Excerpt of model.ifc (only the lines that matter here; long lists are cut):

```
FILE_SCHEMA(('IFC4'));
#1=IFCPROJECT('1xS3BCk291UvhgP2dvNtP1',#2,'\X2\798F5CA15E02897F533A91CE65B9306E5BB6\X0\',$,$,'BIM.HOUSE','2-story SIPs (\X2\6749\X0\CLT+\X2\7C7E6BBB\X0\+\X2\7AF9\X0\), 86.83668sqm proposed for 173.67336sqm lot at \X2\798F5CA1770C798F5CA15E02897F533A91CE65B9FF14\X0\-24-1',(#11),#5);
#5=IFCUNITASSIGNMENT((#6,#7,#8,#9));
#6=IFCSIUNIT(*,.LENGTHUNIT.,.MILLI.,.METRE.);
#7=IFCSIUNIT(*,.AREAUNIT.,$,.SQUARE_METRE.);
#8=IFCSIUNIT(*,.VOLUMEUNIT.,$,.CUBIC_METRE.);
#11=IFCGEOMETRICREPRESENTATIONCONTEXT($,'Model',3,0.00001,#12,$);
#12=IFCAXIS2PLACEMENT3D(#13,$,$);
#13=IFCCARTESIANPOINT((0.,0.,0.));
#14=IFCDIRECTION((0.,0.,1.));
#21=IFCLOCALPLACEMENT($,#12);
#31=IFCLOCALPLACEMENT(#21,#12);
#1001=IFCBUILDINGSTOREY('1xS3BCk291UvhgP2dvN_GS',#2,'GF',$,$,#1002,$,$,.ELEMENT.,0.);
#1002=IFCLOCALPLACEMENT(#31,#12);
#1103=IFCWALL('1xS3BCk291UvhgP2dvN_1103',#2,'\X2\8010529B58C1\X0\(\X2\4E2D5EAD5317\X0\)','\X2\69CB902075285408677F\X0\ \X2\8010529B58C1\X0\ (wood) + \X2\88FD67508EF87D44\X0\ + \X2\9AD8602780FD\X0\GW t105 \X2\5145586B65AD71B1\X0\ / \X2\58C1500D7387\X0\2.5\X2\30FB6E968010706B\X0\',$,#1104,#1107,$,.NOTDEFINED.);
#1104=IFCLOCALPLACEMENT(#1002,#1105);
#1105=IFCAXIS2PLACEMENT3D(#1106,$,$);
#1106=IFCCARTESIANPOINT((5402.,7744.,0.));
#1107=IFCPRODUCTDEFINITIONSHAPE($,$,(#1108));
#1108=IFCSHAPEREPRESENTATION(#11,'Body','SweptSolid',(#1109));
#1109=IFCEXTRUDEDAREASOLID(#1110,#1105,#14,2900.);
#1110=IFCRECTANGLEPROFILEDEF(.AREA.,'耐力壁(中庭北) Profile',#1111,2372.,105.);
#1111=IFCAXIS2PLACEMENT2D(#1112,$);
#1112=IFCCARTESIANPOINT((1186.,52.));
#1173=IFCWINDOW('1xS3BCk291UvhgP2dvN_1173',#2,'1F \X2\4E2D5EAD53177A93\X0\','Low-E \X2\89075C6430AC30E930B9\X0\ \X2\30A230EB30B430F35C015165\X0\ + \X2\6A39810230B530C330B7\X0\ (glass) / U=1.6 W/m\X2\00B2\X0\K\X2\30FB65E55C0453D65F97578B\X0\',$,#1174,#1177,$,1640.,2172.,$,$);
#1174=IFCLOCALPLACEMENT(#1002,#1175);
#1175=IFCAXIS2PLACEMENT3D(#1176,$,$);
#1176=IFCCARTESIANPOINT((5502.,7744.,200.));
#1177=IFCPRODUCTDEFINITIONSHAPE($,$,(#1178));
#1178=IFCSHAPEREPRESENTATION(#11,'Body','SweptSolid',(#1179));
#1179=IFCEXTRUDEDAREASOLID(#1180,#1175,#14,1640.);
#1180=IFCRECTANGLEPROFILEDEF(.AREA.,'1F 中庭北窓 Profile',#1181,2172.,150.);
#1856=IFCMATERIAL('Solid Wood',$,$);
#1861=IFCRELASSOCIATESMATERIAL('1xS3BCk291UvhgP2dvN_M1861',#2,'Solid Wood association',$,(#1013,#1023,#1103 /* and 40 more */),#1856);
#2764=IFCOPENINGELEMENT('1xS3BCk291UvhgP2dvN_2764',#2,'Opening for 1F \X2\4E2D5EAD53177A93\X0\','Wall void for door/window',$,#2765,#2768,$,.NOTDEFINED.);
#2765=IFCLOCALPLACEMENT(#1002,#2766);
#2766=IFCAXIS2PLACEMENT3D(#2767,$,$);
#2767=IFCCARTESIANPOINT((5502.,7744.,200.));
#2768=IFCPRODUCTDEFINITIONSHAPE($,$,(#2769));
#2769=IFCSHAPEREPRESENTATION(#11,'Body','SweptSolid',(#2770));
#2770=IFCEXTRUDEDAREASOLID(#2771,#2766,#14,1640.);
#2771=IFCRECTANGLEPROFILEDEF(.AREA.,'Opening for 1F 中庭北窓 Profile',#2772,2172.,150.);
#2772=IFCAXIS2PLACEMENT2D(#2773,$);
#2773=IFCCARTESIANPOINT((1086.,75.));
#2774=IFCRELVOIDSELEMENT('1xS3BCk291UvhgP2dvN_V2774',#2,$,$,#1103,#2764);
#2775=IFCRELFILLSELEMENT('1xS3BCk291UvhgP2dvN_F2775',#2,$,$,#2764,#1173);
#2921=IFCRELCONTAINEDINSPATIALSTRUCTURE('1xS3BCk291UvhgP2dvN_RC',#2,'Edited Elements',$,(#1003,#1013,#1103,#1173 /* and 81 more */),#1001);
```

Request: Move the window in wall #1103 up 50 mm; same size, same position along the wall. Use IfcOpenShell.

```python
import numpy as np
import ifcopenshell
import ifcopenshell.api.geometry
import ifcopenshell.util.placement
import ifcopenshell.util.unit

model = ifcopenshell.open("model.ifc")
unit_scale = ifcopenshell.util.unit.calculate_unit_scale(model)

window = model.by_id(1173)
opening = window.FillsVoids[0].RelatingOpeningElement
dz = 0.05 / unit_scale

shift = np.array([0.0, 0.0, dz])
# The window is not placed relative to its opening, so move both.
for product in (opening, window):
    matrix = ifcopenshell.util.placement.get_local_placement(product.ObjectPlacement)
    matrix[:3, 3] += shift
    ifcopenshell.api.geometry.edit_object_placement(model, product=product, matrix=matrix, is_si=False)

print(f"moved by {dz * unit_scale:+.3f} m")

model.write("model_edited.ifc")
```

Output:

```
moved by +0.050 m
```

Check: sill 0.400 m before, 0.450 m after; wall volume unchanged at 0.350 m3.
